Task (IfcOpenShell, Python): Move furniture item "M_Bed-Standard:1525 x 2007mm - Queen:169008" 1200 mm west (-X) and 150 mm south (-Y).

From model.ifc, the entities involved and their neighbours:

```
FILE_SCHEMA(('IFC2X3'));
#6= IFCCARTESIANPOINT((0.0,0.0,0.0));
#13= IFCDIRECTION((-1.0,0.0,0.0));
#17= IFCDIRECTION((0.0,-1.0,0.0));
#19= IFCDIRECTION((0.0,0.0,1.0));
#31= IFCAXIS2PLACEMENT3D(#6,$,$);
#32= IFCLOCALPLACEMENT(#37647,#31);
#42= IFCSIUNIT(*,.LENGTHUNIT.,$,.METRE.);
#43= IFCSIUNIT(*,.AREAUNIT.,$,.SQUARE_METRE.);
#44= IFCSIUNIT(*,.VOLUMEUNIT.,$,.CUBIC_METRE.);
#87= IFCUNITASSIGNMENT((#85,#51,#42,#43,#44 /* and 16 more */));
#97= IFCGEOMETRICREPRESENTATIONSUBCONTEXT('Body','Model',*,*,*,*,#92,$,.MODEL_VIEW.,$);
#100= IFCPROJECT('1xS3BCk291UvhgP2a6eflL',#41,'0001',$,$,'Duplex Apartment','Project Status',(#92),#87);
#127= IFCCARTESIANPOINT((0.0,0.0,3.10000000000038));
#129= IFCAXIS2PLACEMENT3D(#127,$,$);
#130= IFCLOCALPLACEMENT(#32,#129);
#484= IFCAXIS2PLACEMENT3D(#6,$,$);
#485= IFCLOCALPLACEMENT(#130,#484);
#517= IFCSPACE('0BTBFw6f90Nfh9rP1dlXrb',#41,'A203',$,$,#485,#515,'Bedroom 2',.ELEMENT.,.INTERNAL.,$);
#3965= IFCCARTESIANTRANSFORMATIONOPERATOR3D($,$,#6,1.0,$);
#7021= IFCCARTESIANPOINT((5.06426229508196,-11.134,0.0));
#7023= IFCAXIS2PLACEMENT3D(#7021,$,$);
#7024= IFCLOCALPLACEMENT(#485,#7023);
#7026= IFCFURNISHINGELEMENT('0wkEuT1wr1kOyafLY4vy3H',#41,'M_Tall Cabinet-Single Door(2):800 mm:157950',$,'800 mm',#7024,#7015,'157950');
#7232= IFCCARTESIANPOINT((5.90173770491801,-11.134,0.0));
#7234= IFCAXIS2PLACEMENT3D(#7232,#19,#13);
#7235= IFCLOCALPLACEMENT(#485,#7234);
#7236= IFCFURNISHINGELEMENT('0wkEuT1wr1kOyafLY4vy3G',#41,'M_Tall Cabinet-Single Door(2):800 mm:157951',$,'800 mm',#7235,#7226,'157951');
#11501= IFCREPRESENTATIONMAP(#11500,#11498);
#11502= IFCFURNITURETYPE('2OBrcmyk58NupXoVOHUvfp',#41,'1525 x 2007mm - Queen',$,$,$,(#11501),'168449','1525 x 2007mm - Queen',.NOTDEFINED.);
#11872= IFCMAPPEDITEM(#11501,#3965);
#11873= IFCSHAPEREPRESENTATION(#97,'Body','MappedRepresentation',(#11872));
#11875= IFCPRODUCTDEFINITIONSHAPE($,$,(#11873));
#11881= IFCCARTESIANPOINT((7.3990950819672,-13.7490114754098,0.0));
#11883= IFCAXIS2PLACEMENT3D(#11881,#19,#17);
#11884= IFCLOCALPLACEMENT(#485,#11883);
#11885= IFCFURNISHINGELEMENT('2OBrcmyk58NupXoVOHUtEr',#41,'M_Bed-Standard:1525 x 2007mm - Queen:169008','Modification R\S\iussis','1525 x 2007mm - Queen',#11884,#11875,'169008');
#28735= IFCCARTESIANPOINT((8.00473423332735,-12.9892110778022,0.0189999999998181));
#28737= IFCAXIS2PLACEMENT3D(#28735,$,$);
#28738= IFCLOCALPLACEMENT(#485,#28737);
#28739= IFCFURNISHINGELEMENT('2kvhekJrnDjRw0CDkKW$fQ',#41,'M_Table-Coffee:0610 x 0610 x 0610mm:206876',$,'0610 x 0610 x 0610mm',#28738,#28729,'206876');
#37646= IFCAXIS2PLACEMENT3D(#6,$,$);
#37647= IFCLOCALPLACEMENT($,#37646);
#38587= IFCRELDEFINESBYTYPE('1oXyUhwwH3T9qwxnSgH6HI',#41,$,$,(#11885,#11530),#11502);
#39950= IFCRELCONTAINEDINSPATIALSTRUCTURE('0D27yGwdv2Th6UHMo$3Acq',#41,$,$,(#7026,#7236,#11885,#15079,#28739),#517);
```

```python
import ifcopenshell
import ifcopenshell.api.geometry
import ifcopenshell.util.placement
import ifcopenshell.util.unit

model = ifcopenshell.open("model.ifc")
unit_scale = ifcopenshell.util.unit.calculate_unit_scale(model)

item = model.by_id(11885)
matrix = ifcopenshell.util.placement.get_local_placement(item.ObjectPlacement)
matrix[0, 3] -= 1.2 / unit_scale
matrix[1, 3] -= 0.15 / unit_scale
ifcopenshell.api.geometry.edit_object_placement(model, product=item, matrix=matrix, is_si=False)

print(ifcopenshell.util.placement.get_local_placement(item.ObjectPlacement).round(3) + 0.0)

model.write("model-out.ifc")
```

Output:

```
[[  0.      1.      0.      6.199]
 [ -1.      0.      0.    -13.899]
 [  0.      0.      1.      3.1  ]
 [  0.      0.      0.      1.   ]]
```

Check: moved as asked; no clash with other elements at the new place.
